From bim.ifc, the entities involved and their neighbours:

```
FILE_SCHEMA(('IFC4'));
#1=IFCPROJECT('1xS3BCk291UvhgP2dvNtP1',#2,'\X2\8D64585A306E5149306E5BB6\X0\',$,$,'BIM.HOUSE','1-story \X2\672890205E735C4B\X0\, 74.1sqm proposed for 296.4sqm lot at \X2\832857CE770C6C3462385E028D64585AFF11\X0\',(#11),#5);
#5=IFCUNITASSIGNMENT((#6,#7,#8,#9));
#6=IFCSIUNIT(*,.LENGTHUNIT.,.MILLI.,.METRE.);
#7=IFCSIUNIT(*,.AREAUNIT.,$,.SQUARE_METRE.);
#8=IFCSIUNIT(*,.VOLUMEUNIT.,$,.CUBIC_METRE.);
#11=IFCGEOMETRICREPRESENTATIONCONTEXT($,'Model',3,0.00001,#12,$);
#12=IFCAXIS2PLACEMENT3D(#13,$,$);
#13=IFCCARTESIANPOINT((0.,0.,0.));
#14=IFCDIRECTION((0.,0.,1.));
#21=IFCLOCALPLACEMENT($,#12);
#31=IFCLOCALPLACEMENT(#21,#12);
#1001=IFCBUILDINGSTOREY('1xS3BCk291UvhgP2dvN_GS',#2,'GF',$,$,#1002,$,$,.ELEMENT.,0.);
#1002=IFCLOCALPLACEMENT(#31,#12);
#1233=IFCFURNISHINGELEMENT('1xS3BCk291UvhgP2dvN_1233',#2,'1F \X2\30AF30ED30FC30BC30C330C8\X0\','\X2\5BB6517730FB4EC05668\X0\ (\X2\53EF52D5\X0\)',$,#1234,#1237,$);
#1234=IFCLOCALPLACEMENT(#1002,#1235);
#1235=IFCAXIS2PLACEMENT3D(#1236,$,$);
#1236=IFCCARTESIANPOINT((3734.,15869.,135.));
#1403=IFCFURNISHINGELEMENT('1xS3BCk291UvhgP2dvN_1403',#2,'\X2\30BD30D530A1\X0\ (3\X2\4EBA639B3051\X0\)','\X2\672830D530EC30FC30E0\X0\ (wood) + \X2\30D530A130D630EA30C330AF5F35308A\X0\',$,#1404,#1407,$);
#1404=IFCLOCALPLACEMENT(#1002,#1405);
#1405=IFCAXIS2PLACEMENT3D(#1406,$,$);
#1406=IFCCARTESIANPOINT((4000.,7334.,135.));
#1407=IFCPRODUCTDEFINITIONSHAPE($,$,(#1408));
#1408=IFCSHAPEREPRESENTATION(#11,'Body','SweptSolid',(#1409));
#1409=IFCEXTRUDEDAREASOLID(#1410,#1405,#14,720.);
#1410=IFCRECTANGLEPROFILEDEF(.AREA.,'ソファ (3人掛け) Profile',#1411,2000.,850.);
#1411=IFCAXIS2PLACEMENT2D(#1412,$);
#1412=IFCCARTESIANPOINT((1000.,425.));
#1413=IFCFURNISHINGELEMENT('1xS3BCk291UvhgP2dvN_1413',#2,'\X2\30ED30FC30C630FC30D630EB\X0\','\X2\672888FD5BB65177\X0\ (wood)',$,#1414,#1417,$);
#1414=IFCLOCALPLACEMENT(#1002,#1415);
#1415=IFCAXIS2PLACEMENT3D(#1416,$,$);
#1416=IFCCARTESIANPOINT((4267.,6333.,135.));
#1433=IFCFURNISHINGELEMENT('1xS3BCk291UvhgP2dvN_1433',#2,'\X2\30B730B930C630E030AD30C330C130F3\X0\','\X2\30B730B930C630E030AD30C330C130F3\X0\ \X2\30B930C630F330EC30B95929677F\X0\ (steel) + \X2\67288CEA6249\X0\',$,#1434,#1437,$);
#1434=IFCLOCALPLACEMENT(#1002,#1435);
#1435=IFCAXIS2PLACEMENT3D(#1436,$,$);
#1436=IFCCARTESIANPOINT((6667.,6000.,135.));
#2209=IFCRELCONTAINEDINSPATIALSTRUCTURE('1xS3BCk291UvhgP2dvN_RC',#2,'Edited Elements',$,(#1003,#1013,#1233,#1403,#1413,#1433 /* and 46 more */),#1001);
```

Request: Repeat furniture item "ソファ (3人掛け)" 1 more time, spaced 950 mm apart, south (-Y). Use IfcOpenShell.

```python
import numpy as np
import ifcopenshell
import ifcopenshell.api.geometry
import ifcopenshell.api.root
import ifcopenshell.util.element
import ifcopenshell.util.placement

model = ifcopenshell.open("bim.ifc")


def reuse_history(source, copy):
    """copy_class also copies each property set's owner history, people and application; keep the originals."""
    for rel in copy.IsDefinedBy:
        if rel.is_a("IfcRelDefinesByProperties") and (history := rel.RelatingPropertyDefinition.OwnerHistory):
            rel.RelatingPropertyDefinition.OwnerHistory = source.OwnerHistory
            ifcopenshell.util.element.remove_deep2(model, history)


source = model.by_id(1403)
base = ifcopenshell.util.placement.get_local_placement(source.ObjectPlacement)
step = np.array([0.0, -1.0, 0.0]) * 950.0

for i in range(1, 2):
    copy = ifcopenshell.api.root.copy_class(model, product=source)
    copy.Representation = ifcopenshell.util.element.copy_deep(
        model, source.Representation, exclude=["IfcGeometricRepresentationContext", "IfcRepresentationMap"]
    )
    reuse_history(source, copy)
    matrix = base.copy()
    matrix[:3, 3] += i * step
    print("added at", matrix[:3, 3].round(3) + 0.0)
    ifcopenshell.api.geometry.edit_object_placement(model, product=copy, matrix=matrix, is_si=False)

model.write("bim-out.ifc")
```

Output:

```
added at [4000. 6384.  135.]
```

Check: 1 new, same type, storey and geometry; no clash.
